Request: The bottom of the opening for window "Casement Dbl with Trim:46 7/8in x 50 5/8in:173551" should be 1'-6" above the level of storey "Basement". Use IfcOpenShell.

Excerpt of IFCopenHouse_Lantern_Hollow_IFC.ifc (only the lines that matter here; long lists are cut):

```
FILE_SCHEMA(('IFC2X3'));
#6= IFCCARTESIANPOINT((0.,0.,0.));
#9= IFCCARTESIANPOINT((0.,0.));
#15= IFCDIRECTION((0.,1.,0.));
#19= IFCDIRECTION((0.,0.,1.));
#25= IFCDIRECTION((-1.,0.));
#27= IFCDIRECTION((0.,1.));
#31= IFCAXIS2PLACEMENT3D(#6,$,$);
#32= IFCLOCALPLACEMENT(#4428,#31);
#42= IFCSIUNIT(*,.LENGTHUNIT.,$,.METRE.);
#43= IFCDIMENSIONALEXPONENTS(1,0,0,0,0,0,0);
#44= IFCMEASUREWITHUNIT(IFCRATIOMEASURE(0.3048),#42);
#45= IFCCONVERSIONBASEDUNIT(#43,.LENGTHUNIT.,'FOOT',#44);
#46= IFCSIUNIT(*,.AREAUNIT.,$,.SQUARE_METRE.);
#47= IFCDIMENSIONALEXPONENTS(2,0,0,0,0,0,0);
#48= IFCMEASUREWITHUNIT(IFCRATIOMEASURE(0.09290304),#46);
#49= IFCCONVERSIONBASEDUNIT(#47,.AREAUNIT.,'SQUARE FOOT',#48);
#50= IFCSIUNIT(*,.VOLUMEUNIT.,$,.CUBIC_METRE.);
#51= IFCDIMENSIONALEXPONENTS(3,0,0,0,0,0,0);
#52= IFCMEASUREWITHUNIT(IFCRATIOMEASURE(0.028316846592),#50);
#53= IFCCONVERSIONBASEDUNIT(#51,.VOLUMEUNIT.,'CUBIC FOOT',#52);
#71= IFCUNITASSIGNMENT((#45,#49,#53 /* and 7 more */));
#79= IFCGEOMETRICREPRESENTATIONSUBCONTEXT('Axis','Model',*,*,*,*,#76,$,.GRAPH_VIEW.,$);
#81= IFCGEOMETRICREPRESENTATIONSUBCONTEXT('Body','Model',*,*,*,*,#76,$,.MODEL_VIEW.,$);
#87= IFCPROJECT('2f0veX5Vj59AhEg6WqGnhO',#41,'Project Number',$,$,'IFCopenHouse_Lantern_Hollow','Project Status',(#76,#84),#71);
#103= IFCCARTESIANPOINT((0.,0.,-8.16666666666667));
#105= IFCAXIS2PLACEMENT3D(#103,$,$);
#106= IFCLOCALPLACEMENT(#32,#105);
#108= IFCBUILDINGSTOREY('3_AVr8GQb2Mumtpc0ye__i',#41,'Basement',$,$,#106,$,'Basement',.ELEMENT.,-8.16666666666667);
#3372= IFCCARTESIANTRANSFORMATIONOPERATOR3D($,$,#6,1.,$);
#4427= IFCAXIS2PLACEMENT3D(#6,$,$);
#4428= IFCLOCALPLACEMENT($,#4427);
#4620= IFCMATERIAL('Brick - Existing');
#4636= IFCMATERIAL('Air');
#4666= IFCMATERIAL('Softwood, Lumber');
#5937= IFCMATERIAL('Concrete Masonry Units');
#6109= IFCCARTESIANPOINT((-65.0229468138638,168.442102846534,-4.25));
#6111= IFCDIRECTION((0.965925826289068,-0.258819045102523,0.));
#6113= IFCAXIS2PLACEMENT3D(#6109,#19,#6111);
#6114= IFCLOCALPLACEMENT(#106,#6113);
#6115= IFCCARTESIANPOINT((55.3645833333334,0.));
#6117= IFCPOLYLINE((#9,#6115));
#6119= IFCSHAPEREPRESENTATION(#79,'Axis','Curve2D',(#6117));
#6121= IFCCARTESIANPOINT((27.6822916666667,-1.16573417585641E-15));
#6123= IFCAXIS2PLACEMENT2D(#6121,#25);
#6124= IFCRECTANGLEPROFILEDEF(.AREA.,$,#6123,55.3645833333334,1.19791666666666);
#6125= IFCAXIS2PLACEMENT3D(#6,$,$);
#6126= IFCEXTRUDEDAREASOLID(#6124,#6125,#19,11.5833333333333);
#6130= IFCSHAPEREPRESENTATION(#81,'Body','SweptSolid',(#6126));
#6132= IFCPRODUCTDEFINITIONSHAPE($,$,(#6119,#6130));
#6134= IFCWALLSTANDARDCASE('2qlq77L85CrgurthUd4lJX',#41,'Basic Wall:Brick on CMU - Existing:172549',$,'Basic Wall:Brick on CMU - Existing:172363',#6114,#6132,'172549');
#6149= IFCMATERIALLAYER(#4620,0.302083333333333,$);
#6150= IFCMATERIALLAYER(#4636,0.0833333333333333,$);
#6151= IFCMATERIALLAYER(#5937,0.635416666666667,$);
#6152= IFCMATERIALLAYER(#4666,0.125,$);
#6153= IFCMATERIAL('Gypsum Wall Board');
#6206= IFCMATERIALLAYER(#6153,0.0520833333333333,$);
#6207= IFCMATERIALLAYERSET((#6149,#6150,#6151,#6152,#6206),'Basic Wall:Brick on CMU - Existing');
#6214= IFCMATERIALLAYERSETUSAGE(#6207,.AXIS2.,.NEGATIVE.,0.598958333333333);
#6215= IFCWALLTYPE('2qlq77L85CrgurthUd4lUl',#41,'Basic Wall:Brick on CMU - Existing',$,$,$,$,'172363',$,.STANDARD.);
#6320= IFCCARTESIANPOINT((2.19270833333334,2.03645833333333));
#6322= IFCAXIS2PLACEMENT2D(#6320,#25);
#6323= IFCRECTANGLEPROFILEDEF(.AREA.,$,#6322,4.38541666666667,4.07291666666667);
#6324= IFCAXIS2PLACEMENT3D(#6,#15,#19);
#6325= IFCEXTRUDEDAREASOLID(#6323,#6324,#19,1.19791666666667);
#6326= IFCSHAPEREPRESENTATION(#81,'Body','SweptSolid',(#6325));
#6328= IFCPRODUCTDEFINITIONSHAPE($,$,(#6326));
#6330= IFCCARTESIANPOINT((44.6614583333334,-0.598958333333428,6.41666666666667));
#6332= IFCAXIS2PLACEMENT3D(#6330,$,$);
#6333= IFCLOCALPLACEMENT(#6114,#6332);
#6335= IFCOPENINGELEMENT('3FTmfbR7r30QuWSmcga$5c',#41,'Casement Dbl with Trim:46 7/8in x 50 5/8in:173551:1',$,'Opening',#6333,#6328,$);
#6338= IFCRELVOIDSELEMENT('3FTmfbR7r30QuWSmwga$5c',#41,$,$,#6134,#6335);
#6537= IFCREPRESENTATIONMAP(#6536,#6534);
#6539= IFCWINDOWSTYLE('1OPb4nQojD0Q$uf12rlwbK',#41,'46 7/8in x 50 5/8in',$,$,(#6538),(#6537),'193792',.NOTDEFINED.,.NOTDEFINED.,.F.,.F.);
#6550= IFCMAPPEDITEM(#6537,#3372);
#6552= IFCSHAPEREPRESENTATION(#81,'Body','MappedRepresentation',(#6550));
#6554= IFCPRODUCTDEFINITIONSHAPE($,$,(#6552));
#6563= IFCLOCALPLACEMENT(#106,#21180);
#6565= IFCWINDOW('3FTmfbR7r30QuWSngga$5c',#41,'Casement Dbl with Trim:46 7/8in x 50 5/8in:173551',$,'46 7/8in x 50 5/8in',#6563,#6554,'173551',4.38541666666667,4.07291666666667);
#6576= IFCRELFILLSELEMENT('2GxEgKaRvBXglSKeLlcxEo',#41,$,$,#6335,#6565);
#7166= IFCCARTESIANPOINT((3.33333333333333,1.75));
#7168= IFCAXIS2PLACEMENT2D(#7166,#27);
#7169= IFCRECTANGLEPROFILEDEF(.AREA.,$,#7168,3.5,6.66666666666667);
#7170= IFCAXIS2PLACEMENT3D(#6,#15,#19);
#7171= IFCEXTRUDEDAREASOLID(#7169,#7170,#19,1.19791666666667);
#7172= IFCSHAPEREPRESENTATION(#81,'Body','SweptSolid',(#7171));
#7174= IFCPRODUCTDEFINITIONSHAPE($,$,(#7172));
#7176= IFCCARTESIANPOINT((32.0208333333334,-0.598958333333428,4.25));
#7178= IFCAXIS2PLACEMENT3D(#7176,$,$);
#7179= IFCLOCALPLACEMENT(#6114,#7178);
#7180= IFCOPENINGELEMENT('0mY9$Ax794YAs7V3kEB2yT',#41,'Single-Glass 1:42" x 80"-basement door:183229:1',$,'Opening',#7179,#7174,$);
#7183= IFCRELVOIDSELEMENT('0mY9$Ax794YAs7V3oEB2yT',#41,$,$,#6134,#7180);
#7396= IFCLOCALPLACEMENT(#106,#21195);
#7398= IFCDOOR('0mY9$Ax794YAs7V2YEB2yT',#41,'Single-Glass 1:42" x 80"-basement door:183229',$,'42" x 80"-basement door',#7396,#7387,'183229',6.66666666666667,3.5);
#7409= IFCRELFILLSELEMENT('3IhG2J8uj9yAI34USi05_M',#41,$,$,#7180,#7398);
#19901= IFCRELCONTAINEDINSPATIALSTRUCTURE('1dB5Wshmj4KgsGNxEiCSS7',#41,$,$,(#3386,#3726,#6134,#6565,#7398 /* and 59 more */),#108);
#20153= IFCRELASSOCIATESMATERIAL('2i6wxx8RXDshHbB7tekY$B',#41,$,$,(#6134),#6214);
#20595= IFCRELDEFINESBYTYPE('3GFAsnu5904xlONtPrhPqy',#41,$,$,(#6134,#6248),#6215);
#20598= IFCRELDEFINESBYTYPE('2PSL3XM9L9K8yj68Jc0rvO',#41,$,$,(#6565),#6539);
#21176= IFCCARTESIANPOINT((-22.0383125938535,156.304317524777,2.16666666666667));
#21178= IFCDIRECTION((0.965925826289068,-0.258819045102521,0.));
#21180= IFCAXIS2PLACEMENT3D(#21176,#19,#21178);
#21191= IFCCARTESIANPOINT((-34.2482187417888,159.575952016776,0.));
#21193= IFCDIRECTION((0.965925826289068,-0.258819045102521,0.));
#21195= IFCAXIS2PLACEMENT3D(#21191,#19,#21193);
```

```python
import numpy as np
import ifcopenshell
import ifcopenshell.api.geometry
import ifcopenshell.geom
import ifcopenshell.util.element
import ifcopenshell.util.placement
import ifcopenshell.util.shape
import ifcopenshell.util.unit

model = ifcopenshell.open("IFCopenHouse_Lantern_Hollow_IFC.ifc")
unit_scale = ifcopenshell.util.unit.calculate_unit_scale(model)

window = model.by_guid("3FTmfbR7r30QuWSngga$5c")
opening = window.FillsVoids[0].RelatingOpeningElement
storey = ifcopenshell.util.element.get_container(window, ifc_class="IfcBuildingStorey")
level = ifcopenshell.util.placement.get_local_placement(storey.ObjectPlacement)[2, 3]

# The opening's origin need not be at the sill, so measure its lowest point.
shape = ifcopenshell.geom.create_shape(ifcopenshell.geom.settings(), opening)
bottom = ifcopenshell.util.shape.get_shape_bottom_elevation(shape, shape.geometry) / unit_scale
dz = level + 18 * 0.0254 / unit_scale - bottom

shift = np.array([0.0, 0.0, dz])
# The window is not placed relative to its opening, so move both.
for product in (opening, window):
    matrix = ifcopenshell.util.placement.get_local_placement(product.ObjectPlacement)
    matrix[:3, 3] += shift
    ifcopenshell.api.geometry.edit_object_placement(model, product=product, matrix=matrix, is_si=False)

print(f"moved by {dz * unit_scale:+.3f} m")

model.write("IFCopenHouse_Lantern_Hollow_IFC_updated.ifc")
```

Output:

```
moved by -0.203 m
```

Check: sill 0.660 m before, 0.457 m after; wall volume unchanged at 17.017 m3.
